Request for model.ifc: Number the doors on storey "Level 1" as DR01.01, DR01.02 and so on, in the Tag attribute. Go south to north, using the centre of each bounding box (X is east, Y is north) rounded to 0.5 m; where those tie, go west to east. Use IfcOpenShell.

First a look at what the model holds.

```python
import ifcopenshell
import ifcopenshell.util.element
import ifcopenshell.util.placement

model = ifcopenshell.open("model.ifc")
print(model.schema)
storey = next(s for s in model.by_type("IfcBuildingStorey") if s.Name == "Level 1")
doors = [e for e in ifcopenshell.util.element.get_decomposition(storey) if e.is_a("IfcDoor")]
for e in sorted(doors, key=lambda e: e.id()):
    origin = ifcopenshell.util.placement.get_local_placement(e.ObjectPlacement)[:3, 3]
    print(e.id(), e.Tag, e.Name, origin.round(2) + 0.0, sep=" | ")
```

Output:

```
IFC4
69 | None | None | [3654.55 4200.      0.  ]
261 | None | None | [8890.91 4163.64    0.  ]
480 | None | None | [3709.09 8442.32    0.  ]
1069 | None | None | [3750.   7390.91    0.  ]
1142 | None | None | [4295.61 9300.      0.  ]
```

```python
import ifcopenshell
import ifcopenshell.geom
import ifcopenshell.util.element
import ifcopenshell.util.shape

model = ifcopenshell.open("model.ifc")
settings = ifcopenshell.geom.settings()
settings.set("use-world-coords", True)


def centre(element):
    shape = ifcopenshell.geom.create_shape(settings, element)
    return ifcopenshell.util.shape.get_bbox_centroid(shape.geometry)


storey = next(s for s in model.by_type("IfcBuildingStorey") if s.Name == "Level 1")
doors = [e for e in ifcopenshell.util.element.get_decomposition(storey) if e.is_a("IfcDoor")]

# Insertion points can sit at a corner or the storey origin, so sort by the geometry (in metres).
centres = {e: centre(e) for e in doors}
doors.sort(key=lambda e: (round(centres[e][1] / 0.5), centres[e][0]))

for i, e in enumerate(doors, start=1):
    number = f"DR01.{i:02d}"
    e.Tag = number
    print(e.id(), number)

model.write("model-out.ifc")
```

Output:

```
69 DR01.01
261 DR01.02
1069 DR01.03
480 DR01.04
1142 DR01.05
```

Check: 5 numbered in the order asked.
